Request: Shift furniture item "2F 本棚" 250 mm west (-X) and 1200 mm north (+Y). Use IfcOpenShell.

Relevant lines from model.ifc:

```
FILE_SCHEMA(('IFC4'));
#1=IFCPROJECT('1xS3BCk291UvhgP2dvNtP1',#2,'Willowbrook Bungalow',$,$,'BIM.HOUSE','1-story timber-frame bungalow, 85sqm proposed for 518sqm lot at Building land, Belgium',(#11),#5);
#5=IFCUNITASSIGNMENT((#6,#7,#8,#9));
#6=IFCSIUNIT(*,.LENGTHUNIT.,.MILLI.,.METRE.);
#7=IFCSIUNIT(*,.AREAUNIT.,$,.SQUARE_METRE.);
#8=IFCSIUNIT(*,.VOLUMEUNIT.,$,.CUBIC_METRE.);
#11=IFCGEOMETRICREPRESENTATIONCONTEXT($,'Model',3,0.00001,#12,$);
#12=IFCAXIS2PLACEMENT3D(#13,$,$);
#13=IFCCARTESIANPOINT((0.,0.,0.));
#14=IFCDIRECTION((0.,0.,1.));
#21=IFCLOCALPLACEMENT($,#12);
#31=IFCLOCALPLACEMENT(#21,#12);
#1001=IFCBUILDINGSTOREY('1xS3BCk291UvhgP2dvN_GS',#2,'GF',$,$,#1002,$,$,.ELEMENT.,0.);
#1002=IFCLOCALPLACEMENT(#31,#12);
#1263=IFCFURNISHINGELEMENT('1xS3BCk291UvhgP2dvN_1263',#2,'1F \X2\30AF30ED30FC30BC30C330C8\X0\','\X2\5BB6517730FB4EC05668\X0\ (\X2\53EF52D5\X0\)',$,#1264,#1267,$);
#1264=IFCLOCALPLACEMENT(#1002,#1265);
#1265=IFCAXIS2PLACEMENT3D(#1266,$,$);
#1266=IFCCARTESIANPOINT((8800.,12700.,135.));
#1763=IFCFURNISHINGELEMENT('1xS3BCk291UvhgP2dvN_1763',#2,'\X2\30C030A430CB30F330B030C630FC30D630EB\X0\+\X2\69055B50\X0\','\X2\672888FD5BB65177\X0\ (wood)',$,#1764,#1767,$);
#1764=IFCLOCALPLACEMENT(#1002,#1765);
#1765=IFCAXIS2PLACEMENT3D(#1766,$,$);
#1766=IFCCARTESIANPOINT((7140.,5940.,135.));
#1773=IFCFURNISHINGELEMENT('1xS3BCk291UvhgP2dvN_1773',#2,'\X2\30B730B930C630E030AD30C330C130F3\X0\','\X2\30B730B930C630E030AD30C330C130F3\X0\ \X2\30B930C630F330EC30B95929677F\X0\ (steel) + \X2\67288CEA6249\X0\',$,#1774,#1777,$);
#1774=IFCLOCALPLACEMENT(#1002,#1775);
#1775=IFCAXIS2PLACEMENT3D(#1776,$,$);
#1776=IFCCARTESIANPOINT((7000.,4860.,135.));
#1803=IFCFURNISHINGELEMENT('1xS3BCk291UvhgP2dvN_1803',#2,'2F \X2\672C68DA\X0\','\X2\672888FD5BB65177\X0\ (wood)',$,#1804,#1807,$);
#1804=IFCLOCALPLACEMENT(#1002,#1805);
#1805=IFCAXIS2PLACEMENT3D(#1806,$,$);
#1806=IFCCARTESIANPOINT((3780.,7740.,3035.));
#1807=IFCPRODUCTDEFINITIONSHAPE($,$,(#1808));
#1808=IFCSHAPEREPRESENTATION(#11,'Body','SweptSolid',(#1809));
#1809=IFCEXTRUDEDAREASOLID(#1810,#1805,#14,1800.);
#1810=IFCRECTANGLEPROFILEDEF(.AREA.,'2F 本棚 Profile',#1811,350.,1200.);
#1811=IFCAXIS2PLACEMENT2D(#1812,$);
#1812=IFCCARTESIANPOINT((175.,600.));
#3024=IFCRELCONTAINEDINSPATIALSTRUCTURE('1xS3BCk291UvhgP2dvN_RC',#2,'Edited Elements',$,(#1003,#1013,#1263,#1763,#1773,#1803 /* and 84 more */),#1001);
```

```python
import ifcopenshell
import ifcopenshell.api.geometry
import ifcopenshell.util.placement

model = ifcopenshell.open("model.ifc")

item = model.by_guid("1xS3BCk291UvhgP2dvN_1803")
matrix = ifcopenshell.util.placement.get_local_placement(item.ObjectPlacement)
matrix[0, 3] -= 250.0
matrix[1, 3] += 1200.0
ifcopenshell.api.geometry.edit_object_placement(model, product=item, matrix=matrix, is_si=False)

print(ifcopenshell.util.placement.get_local_placement(item.ObjectPlacement).round(3) + 0.0)

model.write("model_v2.ifc")
```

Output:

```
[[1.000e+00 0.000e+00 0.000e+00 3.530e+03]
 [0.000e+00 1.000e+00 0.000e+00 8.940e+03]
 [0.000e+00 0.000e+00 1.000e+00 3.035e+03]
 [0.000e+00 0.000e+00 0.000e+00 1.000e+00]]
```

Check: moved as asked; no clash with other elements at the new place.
